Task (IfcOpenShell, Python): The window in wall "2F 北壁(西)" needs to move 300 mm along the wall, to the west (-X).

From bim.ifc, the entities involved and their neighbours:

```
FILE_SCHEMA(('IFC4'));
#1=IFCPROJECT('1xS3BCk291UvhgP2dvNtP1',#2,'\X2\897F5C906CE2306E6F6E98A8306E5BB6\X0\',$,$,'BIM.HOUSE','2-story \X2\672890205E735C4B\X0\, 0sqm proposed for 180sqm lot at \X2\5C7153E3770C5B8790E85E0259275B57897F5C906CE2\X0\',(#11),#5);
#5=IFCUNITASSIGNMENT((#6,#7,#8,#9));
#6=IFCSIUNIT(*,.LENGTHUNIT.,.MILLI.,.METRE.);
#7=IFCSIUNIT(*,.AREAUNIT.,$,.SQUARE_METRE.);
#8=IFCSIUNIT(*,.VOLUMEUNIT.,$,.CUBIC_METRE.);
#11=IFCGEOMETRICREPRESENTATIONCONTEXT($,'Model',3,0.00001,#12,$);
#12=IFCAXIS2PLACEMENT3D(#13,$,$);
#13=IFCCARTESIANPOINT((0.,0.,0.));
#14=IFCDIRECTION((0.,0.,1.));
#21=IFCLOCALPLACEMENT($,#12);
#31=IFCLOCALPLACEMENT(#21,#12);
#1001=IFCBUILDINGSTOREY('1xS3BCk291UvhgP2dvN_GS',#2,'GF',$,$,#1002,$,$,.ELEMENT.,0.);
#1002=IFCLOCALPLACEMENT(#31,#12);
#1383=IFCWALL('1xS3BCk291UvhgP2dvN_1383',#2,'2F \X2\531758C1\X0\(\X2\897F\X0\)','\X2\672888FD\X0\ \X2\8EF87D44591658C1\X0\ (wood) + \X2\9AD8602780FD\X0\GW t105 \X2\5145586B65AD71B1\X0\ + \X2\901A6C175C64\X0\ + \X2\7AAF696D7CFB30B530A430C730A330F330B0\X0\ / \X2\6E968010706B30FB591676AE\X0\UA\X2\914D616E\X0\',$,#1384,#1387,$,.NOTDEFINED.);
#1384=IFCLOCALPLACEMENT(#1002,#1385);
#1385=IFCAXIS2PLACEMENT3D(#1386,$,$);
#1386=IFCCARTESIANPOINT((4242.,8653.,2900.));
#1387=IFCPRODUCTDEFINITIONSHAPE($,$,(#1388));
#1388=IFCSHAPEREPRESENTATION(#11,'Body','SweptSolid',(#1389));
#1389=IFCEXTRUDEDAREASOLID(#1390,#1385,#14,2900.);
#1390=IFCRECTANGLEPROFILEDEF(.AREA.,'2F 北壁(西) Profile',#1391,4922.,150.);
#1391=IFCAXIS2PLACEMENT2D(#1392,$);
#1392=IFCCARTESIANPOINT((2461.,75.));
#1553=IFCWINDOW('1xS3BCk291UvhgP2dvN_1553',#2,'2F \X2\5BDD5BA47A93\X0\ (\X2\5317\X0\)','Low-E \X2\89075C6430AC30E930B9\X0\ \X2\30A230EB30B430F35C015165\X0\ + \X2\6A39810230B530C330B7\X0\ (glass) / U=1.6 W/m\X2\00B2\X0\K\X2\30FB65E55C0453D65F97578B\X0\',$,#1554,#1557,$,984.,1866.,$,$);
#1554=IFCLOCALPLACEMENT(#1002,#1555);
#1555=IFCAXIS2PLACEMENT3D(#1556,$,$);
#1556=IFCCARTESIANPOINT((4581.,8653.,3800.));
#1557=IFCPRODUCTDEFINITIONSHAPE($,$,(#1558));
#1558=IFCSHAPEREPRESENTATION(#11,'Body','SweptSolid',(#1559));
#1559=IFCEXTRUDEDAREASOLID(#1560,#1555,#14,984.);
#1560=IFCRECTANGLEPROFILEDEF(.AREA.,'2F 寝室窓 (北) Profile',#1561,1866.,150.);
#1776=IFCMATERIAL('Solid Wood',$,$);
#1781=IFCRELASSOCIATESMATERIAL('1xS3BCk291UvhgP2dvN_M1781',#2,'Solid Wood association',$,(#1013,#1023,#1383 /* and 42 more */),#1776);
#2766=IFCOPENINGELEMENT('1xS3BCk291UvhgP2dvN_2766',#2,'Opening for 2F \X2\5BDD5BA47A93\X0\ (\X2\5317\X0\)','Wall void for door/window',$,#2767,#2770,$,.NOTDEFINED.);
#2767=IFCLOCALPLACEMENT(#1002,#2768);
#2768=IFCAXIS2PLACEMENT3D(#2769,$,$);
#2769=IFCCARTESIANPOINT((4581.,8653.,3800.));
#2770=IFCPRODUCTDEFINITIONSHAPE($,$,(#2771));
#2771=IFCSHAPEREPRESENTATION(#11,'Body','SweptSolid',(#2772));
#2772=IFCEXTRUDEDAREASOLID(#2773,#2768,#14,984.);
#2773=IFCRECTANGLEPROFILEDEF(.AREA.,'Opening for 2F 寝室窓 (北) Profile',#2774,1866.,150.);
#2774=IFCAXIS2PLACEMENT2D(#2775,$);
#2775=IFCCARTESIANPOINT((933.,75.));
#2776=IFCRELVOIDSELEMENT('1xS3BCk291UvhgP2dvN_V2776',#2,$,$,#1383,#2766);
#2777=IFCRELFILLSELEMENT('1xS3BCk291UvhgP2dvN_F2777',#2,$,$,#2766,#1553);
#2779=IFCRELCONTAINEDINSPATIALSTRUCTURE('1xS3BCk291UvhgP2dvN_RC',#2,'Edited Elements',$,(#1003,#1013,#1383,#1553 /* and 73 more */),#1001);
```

```python
import ifcopenshell
import ifcopenshell.api.geometry
import ifcopenshell.util.placement

model = ifcopenshell.open("bim.ifc")

window = model.by_guid("1xS3BCk291UvhgP2dvN_1553")
opening = window.FillsVoids[0].RelatingOpeningElement
wall = opening.VoidsElements[0].RelatingBuildingElement

wall_matrix = ifcopenshell.util.placement.get_local_placement(wall.ObjectPlacement)
shift = wall_matrix[:3, 0] * -300.0
before = ifcopenshell.util.placement.get_local_placement(window.ObjectPlacement)[:3, 3].copy()

# The window is not placed relative to its opening, so move both.
for product in (opening, window):
    matrix = ifcopenshell.util.placement.get_local_placement(product.ObjectPlacement)
    matrix[:3, 3] += shift
    ifcopenshell.api.geometry.edit_object_placement(model, product=product, matrix=matrix, is_si=False)

after = ifcopenshell.util.placement.get_local_placement(window.ObjectPlacement)[:3, 3]
print("window moved by", (after - before).round(3) + 0.0)

model.write("bim_updated.ifc")
```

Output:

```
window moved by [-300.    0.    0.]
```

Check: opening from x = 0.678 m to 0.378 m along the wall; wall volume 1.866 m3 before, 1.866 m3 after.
